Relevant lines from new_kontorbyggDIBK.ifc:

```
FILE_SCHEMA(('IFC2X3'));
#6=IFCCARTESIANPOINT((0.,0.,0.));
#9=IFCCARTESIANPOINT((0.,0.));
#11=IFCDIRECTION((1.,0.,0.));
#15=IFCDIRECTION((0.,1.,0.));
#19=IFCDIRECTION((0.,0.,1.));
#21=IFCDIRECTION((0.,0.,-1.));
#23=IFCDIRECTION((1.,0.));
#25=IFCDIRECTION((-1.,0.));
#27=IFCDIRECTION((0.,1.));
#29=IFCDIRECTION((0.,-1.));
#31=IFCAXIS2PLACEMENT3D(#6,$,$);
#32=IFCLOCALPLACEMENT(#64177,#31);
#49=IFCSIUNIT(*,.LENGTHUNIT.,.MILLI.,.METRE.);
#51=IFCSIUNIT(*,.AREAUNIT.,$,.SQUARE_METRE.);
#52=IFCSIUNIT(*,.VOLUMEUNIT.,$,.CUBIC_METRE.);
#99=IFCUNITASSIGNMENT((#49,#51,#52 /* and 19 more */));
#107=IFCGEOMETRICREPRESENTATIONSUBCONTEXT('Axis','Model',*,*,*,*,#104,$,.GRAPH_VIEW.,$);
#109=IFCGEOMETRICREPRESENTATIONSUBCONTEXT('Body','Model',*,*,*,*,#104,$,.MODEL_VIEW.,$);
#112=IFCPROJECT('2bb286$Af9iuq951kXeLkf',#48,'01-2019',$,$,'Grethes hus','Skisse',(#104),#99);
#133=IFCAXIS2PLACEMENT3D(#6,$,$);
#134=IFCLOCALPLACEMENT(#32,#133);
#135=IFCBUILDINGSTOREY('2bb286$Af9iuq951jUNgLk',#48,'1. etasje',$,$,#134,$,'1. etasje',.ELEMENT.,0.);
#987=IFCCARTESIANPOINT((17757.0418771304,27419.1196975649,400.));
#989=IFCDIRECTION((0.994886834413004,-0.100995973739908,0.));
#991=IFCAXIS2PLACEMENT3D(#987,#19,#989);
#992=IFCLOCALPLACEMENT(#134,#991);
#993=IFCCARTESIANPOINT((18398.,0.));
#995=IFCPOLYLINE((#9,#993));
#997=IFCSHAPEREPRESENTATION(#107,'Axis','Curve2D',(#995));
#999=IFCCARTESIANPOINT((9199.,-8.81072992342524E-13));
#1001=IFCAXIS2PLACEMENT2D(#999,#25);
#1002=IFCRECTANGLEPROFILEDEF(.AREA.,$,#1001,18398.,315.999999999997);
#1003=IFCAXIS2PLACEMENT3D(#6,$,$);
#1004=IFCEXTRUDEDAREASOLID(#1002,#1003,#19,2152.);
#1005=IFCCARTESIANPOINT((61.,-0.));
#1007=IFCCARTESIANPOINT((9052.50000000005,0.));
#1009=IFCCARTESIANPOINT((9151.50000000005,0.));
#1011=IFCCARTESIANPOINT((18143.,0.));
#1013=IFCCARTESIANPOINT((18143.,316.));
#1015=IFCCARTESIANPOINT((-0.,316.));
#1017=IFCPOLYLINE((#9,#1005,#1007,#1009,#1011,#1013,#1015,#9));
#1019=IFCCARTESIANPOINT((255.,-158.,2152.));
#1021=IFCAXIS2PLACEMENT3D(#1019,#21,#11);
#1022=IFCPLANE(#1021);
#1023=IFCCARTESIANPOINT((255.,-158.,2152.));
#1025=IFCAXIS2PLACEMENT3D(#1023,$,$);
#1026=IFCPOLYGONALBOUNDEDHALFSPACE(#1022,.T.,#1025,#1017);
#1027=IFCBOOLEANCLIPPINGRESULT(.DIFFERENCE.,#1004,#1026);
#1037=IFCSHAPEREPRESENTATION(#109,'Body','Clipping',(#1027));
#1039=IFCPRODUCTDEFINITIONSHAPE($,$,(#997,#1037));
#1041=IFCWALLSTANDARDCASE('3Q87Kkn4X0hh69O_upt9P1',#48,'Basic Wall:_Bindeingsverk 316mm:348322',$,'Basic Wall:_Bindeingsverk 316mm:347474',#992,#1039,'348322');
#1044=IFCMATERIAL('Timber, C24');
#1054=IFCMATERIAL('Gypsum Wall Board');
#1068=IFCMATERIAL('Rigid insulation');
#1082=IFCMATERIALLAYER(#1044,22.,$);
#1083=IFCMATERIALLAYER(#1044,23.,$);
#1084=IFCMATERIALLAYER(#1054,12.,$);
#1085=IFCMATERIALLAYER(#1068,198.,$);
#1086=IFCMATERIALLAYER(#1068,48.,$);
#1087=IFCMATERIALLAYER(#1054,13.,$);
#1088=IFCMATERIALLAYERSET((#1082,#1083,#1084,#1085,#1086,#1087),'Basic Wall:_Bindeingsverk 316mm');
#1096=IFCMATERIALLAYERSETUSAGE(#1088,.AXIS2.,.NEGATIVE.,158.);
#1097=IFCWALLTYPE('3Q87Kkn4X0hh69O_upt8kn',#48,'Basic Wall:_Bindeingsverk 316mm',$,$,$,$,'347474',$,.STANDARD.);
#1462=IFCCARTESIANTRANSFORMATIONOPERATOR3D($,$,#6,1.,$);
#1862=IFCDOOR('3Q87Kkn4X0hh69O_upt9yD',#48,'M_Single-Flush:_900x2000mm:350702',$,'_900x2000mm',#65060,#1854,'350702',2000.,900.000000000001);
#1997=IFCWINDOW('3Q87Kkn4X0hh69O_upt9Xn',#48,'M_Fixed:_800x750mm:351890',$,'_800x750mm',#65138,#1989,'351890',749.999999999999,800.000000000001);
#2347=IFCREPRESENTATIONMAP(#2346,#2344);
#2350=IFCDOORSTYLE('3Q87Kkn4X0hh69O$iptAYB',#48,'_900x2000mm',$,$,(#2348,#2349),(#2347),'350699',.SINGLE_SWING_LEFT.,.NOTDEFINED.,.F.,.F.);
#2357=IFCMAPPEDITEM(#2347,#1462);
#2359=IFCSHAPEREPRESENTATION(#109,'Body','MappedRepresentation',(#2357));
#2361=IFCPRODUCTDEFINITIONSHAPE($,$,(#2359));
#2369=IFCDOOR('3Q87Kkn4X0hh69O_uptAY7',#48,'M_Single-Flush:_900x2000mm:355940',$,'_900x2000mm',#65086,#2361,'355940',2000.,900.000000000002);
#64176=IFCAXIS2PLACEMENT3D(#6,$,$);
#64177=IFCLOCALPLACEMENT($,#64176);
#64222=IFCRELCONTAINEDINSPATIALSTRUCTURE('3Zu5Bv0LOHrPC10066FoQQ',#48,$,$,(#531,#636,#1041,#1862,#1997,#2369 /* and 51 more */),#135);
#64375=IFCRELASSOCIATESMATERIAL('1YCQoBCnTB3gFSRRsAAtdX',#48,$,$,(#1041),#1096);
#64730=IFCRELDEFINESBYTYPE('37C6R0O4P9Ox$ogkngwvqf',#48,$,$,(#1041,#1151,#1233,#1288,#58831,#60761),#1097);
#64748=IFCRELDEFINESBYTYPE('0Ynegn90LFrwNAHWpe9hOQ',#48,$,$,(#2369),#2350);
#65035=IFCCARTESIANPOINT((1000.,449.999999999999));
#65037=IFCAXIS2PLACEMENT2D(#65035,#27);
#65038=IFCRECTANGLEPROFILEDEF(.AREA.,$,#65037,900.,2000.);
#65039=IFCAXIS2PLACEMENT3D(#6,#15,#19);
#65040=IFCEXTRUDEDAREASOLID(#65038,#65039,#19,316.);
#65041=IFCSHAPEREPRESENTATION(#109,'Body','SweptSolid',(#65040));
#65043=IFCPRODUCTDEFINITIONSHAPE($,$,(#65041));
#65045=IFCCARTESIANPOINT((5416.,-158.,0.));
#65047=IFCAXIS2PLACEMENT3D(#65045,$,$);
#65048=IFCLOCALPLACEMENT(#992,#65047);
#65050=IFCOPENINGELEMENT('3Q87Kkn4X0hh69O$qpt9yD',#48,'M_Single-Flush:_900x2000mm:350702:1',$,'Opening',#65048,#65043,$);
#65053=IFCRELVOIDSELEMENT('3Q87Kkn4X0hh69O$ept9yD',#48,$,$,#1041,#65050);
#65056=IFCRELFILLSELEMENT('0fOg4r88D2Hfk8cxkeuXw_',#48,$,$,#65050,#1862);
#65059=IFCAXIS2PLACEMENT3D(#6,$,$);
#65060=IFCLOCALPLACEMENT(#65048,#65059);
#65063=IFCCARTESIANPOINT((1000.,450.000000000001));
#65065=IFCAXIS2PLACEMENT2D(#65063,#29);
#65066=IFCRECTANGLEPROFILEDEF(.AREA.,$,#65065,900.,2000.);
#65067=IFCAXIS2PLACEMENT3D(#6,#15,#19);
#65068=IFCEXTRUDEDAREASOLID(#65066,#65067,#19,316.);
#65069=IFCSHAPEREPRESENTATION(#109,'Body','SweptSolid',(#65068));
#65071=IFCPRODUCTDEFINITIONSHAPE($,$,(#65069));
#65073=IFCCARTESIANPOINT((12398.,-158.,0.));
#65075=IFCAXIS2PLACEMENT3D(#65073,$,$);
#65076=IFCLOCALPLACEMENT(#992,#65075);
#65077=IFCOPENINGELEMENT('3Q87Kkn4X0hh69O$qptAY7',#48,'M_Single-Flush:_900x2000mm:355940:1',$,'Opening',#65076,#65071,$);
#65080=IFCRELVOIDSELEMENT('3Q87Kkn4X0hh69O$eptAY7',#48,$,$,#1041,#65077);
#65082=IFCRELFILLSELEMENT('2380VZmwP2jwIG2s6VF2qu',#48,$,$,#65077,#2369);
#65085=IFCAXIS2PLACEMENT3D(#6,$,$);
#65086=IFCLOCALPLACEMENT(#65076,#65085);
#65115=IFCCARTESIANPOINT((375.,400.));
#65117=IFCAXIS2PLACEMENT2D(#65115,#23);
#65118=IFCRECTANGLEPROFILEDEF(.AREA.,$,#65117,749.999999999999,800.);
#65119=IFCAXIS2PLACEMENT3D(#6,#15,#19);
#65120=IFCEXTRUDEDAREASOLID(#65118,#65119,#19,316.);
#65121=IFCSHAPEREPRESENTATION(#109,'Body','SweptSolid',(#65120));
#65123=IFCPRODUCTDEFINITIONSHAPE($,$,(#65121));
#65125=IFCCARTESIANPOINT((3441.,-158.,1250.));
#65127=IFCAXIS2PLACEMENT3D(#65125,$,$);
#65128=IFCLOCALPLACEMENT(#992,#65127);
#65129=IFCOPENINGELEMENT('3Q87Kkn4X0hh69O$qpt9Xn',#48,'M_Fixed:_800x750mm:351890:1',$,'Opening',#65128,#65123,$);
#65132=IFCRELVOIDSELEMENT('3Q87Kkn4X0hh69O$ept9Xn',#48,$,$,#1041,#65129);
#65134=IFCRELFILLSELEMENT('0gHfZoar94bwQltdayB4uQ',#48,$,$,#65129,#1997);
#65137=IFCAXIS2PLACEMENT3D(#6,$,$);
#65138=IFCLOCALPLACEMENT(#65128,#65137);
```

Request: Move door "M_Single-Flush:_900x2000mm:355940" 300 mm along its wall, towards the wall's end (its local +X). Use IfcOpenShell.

```python
import ifcopenshell
import ifcopenshell.api.geometry
import ifcopenshell.util.placement
import ifcopenshell.util.unit

model = ifcopenshell.open("new_kontorbyggDIBK.ifc")
unit_scale = ifcopenshell.util.unit.calculate_unit_scale(model)

door = model.by_id(2369)
opening = door.FillsVoids[0].RelatingOpeningElement
wall = opening.VoidsElements[0].RelatingBuildingElement

wall_matrix = ifcopenshell.util.placement.get_local_placement(wall.ObjectPlacement)
shift = wall_matrix[:3, 0] * 0.3 / unit_scale
before = ifcopenshell.util.placement.get_local_placement(door.ObjectPlacement)[:3, 3].copy()

# The door is placed relative to its opening, so it follows when the opening moves.
matrix = ifcopenshell.util.placement.get_local_placement(opening.ObjectPlacement)
matrix[:3, 3] += shift
ifcopenshell.api.geometry.edit_object_placement(
    model, product=opening, matrix=matrix, is_si=False, should_transform_children=True
)

after = ifcopenshell.util.placement.get_local_placement(door.ObjectPlacement)[:3, 3]
print("door moved by", (after - before).round(3) + 0.0)

model.write("new_kontorbyggDIBK_updated.ifc")
```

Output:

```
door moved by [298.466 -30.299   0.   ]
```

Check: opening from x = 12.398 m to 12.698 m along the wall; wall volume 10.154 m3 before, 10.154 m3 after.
